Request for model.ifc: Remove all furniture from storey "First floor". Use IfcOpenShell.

First a look at what the model holds.

```python
import ifcopenshell
import ifcopenshell.util.element

model = ifcopenshell.open("model.ifc")
print(model.schema)
storey = next(s for s in model.by_type("IfcBuildingStorey") if s.Name == "First floor")
furniture = [e for e in ifcopenshell.util.element.get_decomposition(storey) if e.is_a("IfcFurnishingElement")]
seen = {}
for e in furniture:
    element_type = ifcopenshell.util.element.get_type(e)
    name = element_type.Name if element_type not in (None, e) else None
    seen[name] = seen.get(name, 0) + 1
for name, count in sorted(seen.items(), key=str):
    print(count, "x", name)
```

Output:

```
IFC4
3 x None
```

```python
import ifcopenshell
import ifcopenshell.api.root
import ifcopenshell.util.element

model = ifcopenshell.open("model.ifc")

storey = next(s for s in model.by_type("IfcBuildingStorey") if s.Name == "First floor")
furniture = [e for e in ifcopenshell.util.element.get_decomposition(storey) if e.is_a("IfcFurnishingElement")]

for e in furniture:
    ifcopenshell.api.root.remove_product(model, product=e)
print(len(furniture), "removed")

model.write("model_updated.ifc")
```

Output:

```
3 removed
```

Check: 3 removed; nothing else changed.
